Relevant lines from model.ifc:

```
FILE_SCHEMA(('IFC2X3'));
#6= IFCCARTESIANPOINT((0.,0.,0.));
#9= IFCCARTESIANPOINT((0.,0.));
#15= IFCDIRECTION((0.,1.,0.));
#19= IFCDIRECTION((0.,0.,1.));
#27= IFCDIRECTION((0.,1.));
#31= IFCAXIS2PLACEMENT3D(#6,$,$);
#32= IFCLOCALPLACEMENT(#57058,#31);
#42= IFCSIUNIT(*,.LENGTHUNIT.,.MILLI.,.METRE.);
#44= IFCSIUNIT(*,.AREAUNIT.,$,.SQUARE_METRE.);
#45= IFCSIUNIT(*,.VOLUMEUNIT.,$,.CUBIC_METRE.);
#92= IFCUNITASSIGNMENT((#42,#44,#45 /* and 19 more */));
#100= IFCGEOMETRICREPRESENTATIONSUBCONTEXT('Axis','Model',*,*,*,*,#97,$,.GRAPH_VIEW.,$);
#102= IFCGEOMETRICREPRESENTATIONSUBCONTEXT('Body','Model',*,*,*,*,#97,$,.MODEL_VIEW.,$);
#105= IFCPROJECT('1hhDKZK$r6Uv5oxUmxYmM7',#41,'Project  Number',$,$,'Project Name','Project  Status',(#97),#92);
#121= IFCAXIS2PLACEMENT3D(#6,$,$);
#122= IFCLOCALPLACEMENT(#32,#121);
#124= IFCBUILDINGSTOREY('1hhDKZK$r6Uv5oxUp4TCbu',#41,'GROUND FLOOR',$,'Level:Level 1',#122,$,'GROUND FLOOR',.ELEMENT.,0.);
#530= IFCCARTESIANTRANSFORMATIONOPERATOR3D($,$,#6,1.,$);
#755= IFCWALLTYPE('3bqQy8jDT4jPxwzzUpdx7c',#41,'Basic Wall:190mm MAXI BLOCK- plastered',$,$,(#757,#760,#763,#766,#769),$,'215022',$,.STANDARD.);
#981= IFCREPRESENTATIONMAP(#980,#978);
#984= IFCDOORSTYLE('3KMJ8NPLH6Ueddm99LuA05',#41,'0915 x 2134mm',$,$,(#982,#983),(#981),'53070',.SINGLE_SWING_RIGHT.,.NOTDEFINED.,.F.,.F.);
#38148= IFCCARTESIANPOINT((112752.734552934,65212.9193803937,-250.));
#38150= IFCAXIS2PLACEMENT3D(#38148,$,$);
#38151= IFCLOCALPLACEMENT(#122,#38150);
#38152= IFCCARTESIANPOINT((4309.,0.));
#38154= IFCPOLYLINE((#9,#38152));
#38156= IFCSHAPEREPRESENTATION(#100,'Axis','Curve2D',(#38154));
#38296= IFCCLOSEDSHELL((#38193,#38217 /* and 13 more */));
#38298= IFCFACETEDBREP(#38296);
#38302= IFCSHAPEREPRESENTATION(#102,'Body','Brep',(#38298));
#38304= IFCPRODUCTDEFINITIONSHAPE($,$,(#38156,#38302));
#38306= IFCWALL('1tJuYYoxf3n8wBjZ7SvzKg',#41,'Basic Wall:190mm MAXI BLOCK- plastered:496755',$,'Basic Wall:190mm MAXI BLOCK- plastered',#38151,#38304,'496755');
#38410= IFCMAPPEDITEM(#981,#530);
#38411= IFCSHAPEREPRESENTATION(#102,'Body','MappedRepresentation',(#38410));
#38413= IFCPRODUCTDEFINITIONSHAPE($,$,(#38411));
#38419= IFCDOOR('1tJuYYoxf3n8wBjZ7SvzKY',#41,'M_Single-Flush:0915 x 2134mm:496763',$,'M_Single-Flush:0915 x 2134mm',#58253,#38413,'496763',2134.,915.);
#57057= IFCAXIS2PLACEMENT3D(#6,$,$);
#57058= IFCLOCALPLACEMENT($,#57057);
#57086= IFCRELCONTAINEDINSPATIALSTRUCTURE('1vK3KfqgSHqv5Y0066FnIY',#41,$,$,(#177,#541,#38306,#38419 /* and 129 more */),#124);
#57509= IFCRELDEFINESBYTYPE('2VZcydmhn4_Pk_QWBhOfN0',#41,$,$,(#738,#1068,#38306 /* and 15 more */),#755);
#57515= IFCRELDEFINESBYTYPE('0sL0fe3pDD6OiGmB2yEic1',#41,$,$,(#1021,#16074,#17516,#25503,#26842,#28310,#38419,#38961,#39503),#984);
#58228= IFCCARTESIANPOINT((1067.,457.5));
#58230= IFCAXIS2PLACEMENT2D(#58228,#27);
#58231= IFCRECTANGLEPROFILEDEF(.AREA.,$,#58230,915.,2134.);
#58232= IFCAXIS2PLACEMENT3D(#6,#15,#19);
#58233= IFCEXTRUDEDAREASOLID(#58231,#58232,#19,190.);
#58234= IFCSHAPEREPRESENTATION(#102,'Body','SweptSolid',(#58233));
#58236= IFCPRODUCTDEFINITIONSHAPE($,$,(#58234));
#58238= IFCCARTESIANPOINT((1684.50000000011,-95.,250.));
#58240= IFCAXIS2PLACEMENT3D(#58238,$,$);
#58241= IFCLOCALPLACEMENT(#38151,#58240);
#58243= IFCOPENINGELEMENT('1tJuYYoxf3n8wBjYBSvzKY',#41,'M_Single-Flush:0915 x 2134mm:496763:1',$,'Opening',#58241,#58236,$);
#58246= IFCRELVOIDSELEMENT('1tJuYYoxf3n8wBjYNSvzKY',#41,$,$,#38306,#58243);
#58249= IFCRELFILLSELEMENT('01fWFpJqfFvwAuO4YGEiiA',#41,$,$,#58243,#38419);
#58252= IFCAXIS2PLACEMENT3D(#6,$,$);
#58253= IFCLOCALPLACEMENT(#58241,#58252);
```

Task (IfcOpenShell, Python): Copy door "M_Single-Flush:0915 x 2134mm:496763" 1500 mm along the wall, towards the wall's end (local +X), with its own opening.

```python
import ifcopenshell
import ifcopenshell.api.feature
import ifcopenshell.api.geometry
import ifcopenshell.api.root
import ifcopenshell.geom
import ifcopenshell.util.element
import ifcopenshell.util.placement
import ifcopenshell.util.shape

model = ifcopenshell.open("model.ifc")
settings = ifcopenshell.geom.settings()


def volume(element):
    """Net volume in cubic metres, openings subtracted."""
    shape = ifcopenshell.geom.create_shape(settings, element)
    return ifcopenshell.util.shape.get_volume(shape.geometry)


def reuse_history(source, copy):
    """copy_class also copies each property set's owner history, people and application; keep the originals."""
    for rel in copy.IsDefinedBy:
        if rel.is_a("IfcRelDefinesByProperties") and (history := rel.RelatingPropertyDefinition.OwnerHistory):
            rel.RelatingPropertyDefinition.OwnerHistory = source.OwnerHistory
            ifcopenshell.util.element.remove_deep2(model, history)


door = model.by_guid("1tJuYYoxf3n8wBjZ7SvzKY")
opening = door.FillsVoids[0].RelatingOpeningElement
wall = opening.VoidsElements[0].RelatingBuildingElement
before = volume(wall)
shift = ifcopenshell.util.placement.get_local_placement(wall.ObjectPlacement)[:3, 0] * 1500.0

# copy_class copies the void relationship, type, container and properties, but no geometry.
new_opening = ifcopenshell.api.root.copy_class(model, product=opening)
new_opening.Representation = ifcopenshell.util.element.copy_deep(
    model, opening.Representation, exclude=["IfcGeometricRepresentationContext", "IfcRepresentationMap"]
)
new_opening.Name = "M_Single-Flush:0915 x 2134mm"
new_door = ifcopenshell.api.root.copy_class(model, product=door)
new_door.Representation = ifcopenshell.util.element.copy_deep(
    model, door.Representation, exclude=["IfcGeometricRepresentationContext", "IfcRepresentationMap"]
)
new_door.Name = "M_Single-Flush:0915 x 2134mm"
new_door.Tag = None
reuse_history(door, new_door)
fills = ifcopenshell.api.feature.add_filling(model, opening=new_opening, element=new_door)
fills.OwnerHistory = new_door.OwnerHistory  # required in IFC2X3

for old, new in ((opening, new_opening), (door, new_door)):
    matrix = ifcopenshell.util.placement.get_local_placement(old.ObjectPlacement)
    matrix[:3, 3] += shift
    ifcopenshell.api.geometry.edit_object_placement(model, product=new, matrix=matrix, is_si=False)

after = volume(wall)

print(f"wall volume {before:.3f} -> {after:.3f} m3")

model.write("model-out.ifc")
```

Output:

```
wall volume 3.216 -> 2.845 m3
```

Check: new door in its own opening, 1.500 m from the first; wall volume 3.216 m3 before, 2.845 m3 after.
